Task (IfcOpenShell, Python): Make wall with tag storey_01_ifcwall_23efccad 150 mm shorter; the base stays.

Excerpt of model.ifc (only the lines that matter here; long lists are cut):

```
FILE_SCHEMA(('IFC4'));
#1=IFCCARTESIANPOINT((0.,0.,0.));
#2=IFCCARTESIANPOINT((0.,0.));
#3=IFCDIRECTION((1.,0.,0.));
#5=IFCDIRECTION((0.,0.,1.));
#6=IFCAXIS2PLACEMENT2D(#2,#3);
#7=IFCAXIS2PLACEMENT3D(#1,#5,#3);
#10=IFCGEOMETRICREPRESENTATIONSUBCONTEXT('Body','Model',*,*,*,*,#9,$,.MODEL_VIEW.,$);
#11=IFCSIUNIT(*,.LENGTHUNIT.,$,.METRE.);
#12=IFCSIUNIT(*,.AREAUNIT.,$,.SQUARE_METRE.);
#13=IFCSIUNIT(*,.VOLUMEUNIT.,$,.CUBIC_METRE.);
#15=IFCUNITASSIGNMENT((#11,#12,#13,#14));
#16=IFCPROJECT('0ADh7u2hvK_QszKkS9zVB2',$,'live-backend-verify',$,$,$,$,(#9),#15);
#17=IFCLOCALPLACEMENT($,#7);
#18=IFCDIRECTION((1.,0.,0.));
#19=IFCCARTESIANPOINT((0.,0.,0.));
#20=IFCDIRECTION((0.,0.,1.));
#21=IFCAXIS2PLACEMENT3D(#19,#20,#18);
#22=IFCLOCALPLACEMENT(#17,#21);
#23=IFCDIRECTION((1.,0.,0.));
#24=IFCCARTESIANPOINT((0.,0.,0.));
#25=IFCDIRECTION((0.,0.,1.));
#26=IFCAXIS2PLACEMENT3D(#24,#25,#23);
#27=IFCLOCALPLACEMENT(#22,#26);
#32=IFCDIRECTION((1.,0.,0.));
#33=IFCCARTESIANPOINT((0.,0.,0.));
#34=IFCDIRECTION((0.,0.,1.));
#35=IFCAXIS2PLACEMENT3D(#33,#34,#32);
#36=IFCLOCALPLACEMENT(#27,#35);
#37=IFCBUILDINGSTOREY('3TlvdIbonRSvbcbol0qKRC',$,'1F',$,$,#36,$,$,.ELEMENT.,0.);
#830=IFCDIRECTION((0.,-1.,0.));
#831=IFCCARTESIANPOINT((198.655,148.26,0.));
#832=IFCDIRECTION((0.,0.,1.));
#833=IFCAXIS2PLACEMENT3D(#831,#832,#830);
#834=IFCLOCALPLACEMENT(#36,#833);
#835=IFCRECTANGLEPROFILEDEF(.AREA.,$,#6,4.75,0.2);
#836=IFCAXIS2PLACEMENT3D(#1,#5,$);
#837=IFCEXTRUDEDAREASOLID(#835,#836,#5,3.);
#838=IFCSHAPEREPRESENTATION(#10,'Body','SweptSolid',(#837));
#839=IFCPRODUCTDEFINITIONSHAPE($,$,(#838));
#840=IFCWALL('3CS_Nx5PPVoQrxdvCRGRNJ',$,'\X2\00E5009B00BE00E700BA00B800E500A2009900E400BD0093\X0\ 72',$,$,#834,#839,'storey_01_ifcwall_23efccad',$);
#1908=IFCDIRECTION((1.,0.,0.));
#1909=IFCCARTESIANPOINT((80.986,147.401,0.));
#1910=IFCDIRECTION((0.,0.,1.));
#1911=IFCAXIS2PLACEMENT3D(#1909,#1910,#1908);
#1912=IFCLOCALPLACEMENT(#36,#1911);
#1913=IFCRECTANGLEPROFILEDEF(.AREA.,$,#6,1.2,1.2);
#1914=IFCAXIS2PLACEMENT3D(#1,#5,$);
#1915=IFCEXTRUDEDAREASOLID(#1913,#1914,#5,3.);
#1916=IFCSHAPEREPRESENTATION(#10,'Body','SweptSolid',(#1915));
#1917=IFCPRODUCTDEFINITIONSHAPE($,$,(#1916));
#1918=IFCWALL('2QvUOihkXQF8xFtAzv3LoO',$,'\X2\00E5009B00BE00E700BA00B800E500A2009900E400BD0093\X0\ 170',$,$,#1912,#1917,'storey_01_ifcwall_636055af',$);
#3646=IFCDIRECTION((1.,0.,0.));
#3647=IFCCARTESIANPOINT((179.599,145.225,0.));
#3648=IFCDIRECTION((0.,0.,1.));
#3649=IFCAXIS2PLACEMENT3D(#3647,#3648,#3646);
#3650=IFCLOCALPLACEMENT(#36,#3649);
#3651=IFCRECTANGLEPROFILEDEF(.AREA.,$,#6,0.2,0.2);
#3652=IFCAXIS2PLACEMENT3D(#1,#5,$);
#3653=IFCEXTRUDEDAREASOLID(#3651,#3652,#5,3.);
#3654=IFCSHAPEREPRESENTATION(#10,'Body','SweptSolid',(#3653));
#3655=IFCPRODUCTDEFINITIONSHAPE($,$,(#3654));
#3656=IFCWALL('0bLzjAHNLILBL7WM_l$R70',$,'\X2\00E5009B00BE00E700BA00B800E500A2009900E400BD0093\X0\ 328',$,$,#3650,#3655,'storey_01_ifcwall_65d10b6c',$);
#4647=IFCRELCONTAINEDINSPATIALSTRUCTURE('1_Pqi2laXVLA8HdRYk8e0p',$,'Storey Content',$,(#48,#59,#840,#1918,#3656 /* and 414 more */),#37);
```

```python
import ifcopenshell
import ifcopenshell.geom
import ifcopenshell.util.representation
import ifcopenshell.util.shape
import ifcopenshell.util.unit

model = ifcopenshell.open("model.ifc")
unit_scale = ifcopenshell.util.unit.calculate_unit_scale(model)
settings = ifcopenshell.geom.settings()


def volume(element):
    """Net volume in cubic metres, openings subtracted."""
    shape = ifcopenshell.geom.create_shape(settings, element)
    return ifcopenshell.util.shape.get_volume(shape.geometry)


wall = model.by_guid("3CS_Nx5PPVoQrxdvCRGRNJ")
before = volume(wall)

body = ifcopenshell.util.representation.get_representation(wall, "Model", "Body")
solid = body.Items[0]
old_height = solid.Depth
solid.Depth -= 0.15 / unit_scale
after = volume(wall)

print(f"height {old_height:g} -> {solid.Depth:g}, volume {before:.3f} -> {after:.3f} m3")

model.write("model_updated.ifc")
```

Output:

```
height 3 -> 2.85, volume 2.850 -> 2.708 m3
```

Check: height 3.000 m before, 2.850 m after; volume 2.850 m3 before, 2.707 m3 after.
